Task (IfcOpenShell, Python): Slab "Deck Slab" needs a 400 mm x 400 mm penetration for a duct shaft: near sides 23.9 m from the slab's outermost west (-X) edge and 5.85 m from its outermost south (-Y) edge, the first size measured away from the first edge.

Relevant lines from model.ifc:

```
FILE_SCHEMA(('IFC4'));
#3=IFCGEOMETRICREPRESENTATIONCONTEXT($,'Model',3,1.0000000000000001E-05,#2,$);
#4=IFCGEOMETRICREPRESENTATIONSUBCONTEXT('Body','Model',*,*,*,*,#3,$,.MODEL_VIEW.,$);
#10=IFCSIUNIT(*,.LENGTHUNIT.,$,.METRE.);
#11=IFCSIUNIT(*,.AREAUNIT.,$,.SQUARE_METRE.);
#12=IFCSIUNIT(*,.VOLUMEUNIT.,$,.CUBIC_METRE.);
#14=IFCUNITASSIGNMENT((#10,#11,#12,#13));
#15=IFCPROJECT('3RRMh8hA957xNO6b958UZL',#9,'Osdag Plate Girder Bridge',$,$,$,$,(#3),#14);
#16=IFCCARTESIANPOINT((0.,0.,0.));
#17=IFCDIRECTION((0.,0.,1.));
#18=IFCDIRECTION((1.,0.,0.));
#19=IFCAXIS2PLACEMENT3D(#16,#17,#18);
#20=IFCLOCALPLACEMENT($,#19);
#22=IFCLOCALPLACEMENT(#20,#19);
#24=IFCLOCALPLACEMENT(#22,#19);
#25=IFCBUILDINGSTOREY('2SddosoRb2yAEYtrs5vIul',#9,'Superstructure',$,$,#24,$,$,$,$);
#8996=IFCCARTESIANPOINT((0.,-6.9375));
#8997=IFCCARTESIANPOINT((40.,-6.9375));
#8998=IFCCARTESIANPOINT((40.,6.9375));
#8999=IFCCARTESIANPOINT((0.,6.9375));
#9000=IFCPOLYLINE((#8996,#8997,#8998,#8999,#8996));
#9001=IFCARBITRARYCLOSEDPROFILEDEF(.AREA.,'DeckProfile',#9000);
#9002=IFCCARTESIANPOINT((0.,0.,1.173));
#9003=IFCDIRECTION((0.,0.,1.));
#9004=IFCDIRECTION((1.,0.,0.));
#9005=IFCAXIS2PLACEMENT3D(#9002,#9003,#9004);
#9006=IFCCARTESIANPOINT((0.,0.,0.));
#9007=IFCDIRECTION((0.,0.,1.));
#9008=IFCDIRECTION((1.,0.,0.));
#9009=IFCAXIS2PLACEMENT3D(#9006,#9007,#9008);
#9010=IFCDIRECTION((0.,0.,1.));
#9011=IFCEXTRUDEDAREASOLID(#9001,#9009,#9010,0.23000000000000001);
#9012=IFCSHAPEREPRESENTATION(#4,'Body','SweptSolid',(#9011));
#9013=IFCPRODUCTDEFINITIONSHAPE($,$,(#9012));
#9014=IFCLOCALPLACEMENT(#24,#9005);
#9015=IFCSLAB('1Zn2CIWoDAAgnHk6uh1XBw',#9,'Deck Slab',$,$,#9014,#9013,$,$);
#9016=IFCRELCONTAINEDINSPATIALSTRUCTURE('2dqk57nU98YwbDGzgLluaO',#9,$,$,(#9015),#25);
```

```python
import numpy as np
import ifcopenshell
import ifcopenshell.api.feature
import ifcopenshell.api.geometry
import ifcopenshell.api.root
import ifcopenshell.geom
import ifcopenshell.util.placement
import ifcopenshell.util.representation
import ifcopenshell.util.shape
import ifcopenshell.util.unit

model = ifcopenshell.open("model.ifc")
unit_scale = ifcopenshell.util.unit.calculate_unit_scale(model)
settings = ifcopenshell.geom.settings()


def volume(element):
    """Net volume in cubic metres, openings subtracted."""
    shape = ifcopenshell.geom.create_shape(settings, element)
    return ifcopenshell.util.shape.get_volume(shape.geometry)


slab = model.by_guid("1Zn2CIWoDAAgnHk6uh1XBw")
before = volume(slab)

# Extent in the slab's own axes, in metres. The edges named are its -X and -Y sides.
slab_shape = ifcopenshell.geom.create_shape(settings, slab)
vertices = ifcopenshell.util.shape.get_vertices(slab_shape.geometry)
x_min, y_min, bottom = vertices.min(axis=0)
top = vertices[:, 2].max()

opening = ifcopenshell.api.root.create_entity(model, ifc_class="IfcOpeningElement", name="Duct shaft opening", predefined_type="OPENING")
context = ifcopenshell.util.representation.get_context(model, "Model", "Body", "MODEL_VIEW")
width, depth = 0.4, 0.4
outline = [(0.0, 0.0), (width, 0.0), (width, depth), (0.0, depth), (0.0, 0.0)]
# Overshoot both faces by 50 mm so the cut is clean.
shape = ifcopenshell.api.geometry.add_slab_representation(
    model, context=context, depth=top - bottom + 0.1, polyline=outline
)
ifcopenshell.api.geometry.assign_representation(model, product=opening, representation=shape)

matrix = ifcopenshell.util.placement.get_local_placement(slab.ObjectPlacement)
matrix[:, 3] = matrix @ np.append(np.array([x_min + 23.9, y_min + 5.85, bottom - 0.05]) / unit_scale, 1.0)
ifcopenshell.api.geometry.edit_object_placement(model, product=opening, matrix=matrix, is_si=False)
ifcopenshell.api.feature.add_feature(model, feature=opening, element=slab)

after = volume(slab)

print(f"slab volume {before:.3f} -> {after:.3f} m3")

model.write("model_edited.ifc")
```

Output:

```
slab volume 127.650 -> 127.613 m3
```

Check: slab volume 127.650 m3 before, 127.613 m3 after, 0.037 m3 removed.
